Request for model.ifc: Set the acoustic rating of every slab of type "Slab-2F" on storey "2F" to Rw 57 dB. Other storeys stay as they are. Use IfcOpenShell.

First a look at what the model holds.

```python
import ifcopenshell
import ifcopenshell.util.element

model = ifcopenshell.open("model.ifc")
print(model.schema)
storey = next(s for s in model.by_type("IfcBuildingStorey") if s.Name == "2F")
slabs = [e for e in ifcopenshell.util.element.get_decomposition(storey) if e.is_a("IfcSlab")]
seen = {}
for e in slabs:
    element_type = ifcopenshell.util.element.get_type(e)
    key = (element_type.Name if element_type != e and element_type else None, ifcopenshell.util.element.get_pset(e, "Pset_SlabCommon", "AcousticRating"))
    seen[key] = seen.get(key, 0) + 1
for (name, value), count in sorted(seen.items(), key=str):
    print(count, "x", name, "|", value)
```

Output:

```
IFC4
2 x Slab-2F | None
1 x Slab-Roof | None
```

```python
import ifcopenshell
import ifcopenshell.api.pset
import ifcopenshell.util.element

model = ifcopenshell.open("model.ifc")

storey = next(s for s in model.by_type("IfcBuildingStorey") if s.Name == "2F")
slabs = [e for e in ifcopenshell.util.element.get_decomposition(storey) if e.is_a("IfcSlab")]

count = 0
for e in slabs:
    element_type = ifcopenshell.util.element.get_type(e)
    if element_type in (None, e) or element_type.Name != "Slab-2F":
        continue
    # add_pset returns the element's existing set when there is one.
    pset = ifcopenshell.api.pset.add_pset(model, product=e, name="Pset_SlabCommon")
    ifcopenshell.api.pset.edit_pset(model, pset=pset, properties={"AcousticRating": "Rw 57 dB"})
    count += 1

print(count, "slabs updated")

model.write("model_updated.ifc")
```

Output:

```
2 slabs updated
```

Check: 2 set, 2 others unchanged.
